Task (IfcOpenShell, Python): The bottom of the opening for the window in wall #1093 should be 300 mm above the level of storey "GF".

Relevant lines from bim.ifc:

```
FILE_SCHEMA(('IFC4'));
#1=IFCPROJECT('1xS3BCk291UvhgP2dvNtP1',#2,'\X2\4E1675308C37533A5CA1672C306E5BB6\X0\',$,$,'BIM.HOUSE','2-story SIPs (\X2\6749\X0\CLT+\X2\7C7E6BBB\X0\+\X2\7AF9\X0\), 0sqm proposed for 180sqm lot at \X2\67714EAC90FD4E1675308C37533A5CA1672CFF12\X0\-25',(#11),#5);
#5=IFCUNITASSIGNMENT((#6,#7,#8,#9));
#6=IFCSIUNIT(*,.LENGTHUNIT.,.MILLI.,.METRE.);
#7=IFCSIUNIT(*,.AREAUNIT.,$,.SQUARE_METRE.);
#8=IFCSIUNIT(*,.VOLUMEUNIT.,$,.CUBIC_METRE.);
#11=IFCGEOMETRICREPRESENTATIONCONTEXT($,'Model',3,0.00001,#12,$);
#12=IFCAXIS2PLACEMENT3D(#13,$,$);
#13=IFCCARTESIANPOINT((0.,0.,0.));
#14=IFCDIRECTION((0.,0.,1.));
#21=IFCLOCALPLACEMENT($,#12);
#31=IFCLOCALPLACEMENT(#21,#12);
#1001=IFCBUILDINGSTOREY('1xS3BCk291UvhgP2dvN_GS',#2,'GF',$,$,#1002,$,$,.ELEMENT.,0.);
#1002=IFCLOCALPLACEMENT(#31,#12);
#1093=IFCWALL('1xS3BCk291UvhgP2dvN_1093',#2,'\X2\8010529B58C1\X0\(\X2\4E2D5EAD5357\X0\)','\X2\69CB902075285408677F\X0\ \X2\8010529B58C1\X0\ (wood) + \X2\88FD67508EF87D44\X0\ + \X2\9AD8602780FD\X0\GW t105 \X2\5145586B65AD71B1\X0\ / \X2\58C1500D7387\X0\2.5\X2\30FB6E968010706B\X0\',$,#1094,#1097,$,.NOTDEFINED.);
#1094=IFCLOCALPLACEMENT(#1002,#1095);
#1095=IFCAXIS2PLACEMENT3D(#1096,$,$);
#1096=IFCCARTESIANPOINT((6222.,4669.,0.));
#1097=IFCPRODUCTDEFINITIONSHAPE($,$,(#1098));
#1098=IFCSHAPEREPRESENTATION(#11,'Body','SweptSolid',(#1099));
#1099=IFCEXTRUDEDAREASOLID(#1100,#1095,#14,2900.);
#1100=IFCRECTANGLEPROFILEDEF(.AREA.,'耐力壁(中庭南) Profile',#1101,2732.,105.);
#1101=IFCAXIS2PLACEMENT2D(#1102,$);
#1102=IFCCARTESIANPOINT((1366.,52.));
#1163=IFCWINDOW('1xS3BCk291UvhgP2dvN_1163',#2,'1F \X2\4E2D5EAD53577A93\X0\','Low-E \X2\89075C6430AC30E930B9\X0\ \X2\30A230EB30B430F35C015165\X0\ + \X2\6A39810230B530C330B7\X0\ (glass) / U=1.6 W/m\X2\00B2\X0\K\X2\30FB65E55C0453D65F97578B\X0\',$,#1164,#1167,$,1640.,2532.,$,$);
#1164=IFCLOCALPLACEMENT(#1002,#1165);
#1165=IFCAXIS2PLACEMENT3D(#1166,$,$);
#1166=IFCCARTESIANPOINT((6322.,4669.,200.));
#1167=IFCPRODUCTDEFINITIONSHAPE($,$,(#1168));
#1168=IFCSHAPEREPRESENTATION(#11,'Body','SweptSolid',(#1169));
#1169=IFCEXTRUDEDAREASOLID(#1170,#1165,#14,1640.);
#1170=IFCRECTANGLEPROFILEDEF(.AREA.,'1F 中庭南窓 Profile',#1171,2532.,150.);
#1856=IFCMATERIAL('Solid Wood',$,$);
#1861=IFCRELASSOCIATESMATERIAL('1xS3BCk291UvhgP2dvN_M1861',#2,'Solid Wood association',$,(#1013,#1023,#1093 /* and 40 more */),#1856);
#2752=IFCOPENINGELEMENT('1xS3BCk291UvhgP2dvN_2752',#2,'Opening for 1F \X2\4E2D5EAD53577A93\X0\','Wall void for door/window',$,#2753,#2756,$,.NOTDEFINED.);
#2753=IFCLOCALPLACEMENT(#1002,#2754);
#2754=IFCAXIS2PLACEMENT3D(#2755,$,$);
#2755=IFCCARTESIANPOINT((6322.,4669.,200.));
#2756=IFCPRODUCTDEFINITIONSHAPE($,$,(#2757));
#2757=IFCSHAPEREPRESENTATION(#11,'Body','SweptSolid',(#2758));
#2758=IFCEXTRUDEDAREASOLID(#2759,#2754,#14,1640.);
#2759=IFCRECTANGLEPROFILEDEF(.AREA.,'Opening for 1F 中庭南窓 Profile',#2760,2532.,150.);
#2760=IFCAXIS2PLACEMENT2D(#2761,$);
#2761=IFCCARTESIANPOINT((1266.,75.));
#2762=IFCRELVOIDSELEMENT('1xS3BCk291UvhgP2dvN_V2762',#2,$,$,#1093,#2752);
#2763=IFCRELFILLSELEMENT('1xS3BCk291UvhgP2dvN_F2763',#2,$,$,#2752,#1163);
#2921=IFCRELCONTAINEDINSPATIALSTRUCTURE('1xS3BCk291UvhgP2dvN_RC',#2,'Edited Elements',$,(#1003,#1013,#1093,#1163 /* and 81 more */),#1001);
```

```python
import numpy as np
import ifcopenshell
import ifcopenshell.api.geometry
import ifcopenshell.geom
import ifcopenshell.util.element
import ifcopenshell.util.placement
import ifcopenshell.util.shape
import ifcopenshell.util.unit

model = ifcopenshell.open("bim.ifc")
unit_scale = ifcopenshell.util.unit.calculate_unit_scale(model)

window = model.by_guid("1xS3BCk291UvhgP2dvN_1163")
opening = window.FillsVoids[0].RelatingOpeningElement
storey = ifcopenshell.util.element.get_container(window, ifc_class="IfcBuildingStorey")
level = ifcopenshell.util.placement.get_local_placement(storey.ObjectPlacement)[2, 3]

# The opening's origin need not be at the sill, so measure its lowest point.
shape = ifcopenshell.geom.create_shape(ifcopenshell.geom.settings(), opening)
bottom = ifcopenshell.util.shape.get_shape_bottom_elevation(shape, shape.geometry) / unit_scale
dz = level + 0.3 / unit_scale - bottom

shift = np.array([0.0, 0.0, dz])
# The window is not placed relative to its opening, so move both.
for product in (opening, window):
    matrix = ifcopenshell.util.placement.get_local_placement(product.ObjectPlacement)
    matrix[:3, 3] += shift
    ifcopenshell.api.geometry.edit_object_placement(model, product=product, matrix=matrix, is_si=False)

print(f"moved by {dz * unit_scale:+.3f} m")

model.write("bim-out.ifc")
```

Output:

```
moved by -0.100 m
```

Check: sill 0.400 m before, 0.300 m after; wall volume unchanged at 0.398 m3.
